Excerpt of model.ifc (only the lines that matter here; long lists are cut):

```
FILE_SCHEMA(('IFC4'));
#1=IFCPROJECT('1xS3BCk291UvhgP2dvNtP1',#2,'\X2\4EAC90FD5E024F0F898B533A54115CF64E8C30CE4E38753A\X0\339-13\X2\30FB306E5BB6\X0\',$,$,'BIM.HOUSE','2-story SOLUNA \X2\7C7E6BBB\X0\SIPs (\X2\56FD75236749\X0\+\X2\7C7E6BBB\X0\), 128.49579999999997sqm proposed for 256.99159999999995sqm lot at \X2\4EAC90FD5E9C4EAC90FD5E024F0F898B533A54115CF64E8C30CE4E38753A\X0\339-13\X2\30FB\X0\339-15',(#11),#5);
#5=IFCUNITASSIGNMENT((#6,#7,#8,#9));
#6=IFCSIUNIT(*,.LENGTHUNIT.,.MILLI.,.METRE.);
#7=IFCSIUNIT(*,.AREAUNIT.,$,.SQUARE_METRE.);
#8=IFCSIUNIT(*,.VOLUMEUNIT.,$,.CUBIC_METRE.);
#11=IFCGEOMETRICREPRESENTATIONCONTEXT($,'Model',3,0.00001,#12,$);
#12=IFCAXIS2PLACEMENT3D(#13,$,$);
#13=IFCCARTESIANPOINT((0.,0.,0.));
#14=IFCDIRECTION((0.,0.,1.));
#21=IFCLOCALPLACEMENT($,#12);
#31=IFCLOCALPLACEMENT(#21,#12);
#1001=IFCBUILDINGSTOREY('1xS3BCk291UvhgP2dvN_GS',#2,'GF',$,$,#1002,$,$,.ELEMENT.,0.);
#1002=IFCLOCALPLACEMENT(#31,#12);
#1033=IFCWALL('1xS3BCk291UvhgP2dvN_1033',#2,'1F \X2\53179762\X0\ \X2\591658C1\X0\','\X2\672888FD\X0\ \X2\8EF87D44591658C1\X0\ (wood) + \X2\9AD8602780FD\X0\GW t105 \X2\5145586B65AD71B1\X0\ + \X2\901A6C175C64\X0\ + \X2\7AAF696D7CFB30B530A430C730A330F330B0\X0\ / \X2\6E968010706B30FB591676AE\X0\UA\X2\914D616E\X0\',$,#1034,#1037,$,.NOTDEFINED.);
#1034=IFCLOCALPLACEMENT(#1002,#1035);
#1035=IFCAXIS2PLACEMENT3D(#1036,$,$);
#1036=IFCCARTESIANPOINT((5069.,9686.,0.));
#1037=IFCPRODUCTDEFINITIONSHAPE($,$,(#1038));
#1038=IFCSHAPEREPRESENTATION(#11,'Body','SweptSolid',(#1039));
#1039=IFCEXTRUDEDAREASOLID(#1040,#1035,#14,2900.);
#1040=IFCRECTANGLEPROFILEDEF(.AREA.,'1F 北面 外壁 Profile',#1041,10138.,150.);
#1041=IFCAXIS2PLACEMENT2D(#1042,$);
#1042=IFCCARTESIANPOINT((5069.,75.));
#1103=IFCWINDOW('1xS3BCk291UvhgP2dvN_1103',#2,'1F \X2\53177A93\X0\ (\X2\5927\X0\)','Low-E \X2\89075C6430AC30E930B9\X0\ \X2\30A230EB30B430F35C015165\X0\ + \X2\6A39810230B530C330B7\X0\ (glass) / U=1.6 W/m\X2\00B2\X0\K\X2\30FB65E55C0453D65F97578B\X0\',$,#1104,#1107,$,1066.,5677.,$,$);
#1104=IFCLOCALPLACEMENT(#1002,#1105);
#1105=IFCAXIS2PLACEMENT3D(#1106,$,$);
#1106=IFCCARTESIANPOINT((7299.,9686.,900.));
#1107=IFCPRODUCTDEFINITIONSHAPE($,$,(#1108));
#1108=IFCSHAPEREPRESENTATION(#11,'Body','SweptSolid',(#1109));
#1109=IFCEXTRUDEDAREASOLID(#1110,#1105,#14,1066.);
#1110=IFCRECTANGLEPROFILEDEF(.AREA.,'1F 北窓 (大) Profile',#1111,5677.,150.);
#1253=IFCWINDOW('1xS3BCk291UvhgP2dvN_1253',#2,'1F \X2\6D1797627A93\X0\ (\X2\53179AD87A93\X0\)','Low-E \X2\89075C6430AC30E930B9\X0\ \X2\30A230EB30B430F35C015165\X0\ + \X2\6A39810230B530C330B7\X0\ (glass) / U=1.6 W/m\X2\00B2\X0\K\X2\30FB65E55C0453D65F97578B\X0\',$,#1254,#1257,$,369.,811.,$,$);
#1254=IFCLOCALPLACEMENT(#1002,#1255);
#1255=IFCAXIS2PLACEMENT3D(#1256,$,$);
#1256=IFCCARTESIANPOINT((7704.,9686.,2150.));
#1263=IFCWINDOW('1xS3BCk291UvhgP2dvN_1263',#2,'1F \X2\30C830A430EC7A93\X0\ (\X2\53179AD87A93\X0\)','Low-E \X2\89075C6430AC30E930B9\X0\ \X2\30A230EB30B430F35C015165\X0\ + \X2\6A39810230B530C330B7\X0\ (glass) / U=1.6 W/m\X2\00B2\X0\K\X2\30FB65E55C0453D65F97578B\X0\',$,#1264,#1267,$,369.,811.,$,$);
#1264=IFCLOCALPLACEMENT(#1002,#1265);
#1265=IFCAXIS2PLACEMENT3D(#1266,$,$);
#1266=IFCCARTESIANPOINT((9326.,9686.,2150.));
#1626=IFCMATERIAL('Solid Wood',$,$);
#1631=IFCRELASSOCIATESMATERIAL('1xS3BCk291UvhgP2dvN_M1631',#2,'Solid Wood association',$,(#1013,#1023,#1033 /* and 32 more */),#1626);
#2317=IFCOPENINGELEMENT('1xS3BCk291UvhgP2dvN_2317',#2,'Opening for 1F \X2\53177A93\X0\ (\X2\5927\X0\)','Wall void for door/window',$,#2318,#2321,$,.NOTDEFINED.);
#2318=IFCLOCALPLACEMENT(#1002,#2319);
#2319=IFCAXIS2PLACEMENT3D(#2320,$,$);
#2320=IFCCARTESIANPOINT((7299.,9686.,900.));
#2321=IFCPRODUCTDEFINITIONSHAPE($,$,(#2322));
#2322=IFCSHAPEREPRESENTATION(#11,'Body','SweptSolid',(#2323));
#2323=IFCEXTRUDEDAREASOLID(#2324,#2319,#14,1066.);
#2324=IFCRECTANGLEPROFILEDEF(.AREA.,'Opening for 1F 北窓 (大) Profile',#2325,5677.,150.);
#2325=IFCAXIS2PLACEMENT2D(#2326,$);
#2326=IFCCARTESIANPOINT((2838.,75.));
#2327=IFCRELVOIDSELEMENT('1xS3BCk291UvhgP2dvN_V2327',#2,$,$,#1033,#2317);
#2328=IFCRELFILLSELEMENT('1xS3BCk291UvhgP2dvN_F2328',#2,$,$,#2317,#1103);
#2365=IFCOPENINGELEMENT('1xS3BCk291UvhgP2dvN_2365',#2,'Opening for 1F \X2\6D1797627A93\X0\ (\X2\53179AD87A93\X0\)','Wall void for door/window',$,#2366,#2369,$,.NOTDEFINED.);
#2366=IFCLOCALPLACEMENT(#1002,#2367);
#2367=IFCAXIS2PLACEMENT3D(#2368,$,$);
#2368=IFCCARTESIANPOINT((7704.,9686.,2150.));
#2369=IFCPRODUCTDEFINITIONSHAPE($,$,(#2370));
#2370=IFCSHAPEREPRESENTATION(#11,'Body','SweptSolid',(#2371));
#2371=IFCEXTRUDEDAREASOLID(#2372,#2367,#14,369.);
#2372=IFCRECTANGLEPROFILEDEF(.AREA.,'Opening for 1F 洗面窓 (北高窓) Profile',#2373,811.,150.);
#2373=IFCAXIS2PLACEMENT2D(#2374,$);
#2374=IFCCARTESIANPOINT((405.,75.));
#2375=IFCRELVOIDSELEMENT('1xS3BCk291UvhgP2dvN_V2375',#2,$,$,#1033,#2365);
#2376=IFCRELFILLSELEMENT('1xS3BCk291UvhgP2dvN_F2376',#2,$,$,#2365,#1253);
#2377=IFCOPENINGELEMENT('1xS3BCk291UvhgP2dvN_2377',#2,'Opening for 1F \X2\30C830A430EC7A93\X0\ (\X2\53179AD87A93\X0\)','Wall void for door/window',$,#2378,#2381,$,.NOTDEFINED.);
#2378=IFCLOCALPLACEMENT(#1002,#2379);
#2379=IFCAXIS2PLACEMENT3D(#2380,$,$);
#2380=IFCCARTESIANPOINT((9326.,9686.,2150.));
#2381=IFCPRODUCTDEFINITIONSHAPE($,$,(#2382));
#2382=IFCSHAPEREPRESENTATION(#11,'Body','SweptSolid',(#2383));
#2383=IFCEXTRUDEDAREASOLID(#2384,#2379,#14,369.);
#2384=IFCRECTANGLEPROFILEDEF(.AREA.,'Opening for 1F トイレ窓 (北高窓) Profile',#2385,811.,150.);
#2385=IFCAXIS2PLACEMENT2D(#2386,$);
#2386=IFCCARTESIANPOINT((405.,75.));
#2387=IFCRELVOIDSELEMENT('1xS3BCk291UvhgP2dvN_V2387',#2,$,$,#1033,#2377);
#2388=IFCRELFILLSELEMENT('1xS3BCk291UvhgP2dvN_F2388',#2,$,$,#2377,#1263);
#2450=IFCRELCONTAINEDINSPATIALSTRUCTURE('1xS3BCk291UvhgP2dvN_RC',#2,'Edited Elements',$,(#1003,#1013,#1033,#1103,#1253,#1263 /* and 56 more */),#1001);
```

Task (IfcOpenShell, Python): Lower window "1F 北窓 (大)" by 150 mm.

```python
import numpy as np
import ifcopenshell
import ifcopenshell.api.geometry
import ifcopenshell.util.placement
import ifcopenshell.util.unit

model = ifcopenshell.open("model.ifc")
unit_scale = ifcopenshell.util.unit.calculate_unit_scale(model)

window = model.by_guid("1xS3BCk291UvhgP2dvN_1103")
opening = window.FillsVoids[0].RelatingOpeningElement
dz = -0.15 / unit_scale

shift = np.array([0.0, 0.0, dz])
# The window is not placed relative to its opening, so move both.
for product in (opening, window):
    matrix = ifcopenshell.util.placement.get_local_placement(product.ObjectPlacement)
    matrix[:3, 3] += shift
    ifcopenshell.api.geometry.edit_object_placement(model, product=product, matrix=matrix, is_si=False)

print(f"moved by {dz * unit_scale:+.3f} m")

model.write("model_edited.ifc")
```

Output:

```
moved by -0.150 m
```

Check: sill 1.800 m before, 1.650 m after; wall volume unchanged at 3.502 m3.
